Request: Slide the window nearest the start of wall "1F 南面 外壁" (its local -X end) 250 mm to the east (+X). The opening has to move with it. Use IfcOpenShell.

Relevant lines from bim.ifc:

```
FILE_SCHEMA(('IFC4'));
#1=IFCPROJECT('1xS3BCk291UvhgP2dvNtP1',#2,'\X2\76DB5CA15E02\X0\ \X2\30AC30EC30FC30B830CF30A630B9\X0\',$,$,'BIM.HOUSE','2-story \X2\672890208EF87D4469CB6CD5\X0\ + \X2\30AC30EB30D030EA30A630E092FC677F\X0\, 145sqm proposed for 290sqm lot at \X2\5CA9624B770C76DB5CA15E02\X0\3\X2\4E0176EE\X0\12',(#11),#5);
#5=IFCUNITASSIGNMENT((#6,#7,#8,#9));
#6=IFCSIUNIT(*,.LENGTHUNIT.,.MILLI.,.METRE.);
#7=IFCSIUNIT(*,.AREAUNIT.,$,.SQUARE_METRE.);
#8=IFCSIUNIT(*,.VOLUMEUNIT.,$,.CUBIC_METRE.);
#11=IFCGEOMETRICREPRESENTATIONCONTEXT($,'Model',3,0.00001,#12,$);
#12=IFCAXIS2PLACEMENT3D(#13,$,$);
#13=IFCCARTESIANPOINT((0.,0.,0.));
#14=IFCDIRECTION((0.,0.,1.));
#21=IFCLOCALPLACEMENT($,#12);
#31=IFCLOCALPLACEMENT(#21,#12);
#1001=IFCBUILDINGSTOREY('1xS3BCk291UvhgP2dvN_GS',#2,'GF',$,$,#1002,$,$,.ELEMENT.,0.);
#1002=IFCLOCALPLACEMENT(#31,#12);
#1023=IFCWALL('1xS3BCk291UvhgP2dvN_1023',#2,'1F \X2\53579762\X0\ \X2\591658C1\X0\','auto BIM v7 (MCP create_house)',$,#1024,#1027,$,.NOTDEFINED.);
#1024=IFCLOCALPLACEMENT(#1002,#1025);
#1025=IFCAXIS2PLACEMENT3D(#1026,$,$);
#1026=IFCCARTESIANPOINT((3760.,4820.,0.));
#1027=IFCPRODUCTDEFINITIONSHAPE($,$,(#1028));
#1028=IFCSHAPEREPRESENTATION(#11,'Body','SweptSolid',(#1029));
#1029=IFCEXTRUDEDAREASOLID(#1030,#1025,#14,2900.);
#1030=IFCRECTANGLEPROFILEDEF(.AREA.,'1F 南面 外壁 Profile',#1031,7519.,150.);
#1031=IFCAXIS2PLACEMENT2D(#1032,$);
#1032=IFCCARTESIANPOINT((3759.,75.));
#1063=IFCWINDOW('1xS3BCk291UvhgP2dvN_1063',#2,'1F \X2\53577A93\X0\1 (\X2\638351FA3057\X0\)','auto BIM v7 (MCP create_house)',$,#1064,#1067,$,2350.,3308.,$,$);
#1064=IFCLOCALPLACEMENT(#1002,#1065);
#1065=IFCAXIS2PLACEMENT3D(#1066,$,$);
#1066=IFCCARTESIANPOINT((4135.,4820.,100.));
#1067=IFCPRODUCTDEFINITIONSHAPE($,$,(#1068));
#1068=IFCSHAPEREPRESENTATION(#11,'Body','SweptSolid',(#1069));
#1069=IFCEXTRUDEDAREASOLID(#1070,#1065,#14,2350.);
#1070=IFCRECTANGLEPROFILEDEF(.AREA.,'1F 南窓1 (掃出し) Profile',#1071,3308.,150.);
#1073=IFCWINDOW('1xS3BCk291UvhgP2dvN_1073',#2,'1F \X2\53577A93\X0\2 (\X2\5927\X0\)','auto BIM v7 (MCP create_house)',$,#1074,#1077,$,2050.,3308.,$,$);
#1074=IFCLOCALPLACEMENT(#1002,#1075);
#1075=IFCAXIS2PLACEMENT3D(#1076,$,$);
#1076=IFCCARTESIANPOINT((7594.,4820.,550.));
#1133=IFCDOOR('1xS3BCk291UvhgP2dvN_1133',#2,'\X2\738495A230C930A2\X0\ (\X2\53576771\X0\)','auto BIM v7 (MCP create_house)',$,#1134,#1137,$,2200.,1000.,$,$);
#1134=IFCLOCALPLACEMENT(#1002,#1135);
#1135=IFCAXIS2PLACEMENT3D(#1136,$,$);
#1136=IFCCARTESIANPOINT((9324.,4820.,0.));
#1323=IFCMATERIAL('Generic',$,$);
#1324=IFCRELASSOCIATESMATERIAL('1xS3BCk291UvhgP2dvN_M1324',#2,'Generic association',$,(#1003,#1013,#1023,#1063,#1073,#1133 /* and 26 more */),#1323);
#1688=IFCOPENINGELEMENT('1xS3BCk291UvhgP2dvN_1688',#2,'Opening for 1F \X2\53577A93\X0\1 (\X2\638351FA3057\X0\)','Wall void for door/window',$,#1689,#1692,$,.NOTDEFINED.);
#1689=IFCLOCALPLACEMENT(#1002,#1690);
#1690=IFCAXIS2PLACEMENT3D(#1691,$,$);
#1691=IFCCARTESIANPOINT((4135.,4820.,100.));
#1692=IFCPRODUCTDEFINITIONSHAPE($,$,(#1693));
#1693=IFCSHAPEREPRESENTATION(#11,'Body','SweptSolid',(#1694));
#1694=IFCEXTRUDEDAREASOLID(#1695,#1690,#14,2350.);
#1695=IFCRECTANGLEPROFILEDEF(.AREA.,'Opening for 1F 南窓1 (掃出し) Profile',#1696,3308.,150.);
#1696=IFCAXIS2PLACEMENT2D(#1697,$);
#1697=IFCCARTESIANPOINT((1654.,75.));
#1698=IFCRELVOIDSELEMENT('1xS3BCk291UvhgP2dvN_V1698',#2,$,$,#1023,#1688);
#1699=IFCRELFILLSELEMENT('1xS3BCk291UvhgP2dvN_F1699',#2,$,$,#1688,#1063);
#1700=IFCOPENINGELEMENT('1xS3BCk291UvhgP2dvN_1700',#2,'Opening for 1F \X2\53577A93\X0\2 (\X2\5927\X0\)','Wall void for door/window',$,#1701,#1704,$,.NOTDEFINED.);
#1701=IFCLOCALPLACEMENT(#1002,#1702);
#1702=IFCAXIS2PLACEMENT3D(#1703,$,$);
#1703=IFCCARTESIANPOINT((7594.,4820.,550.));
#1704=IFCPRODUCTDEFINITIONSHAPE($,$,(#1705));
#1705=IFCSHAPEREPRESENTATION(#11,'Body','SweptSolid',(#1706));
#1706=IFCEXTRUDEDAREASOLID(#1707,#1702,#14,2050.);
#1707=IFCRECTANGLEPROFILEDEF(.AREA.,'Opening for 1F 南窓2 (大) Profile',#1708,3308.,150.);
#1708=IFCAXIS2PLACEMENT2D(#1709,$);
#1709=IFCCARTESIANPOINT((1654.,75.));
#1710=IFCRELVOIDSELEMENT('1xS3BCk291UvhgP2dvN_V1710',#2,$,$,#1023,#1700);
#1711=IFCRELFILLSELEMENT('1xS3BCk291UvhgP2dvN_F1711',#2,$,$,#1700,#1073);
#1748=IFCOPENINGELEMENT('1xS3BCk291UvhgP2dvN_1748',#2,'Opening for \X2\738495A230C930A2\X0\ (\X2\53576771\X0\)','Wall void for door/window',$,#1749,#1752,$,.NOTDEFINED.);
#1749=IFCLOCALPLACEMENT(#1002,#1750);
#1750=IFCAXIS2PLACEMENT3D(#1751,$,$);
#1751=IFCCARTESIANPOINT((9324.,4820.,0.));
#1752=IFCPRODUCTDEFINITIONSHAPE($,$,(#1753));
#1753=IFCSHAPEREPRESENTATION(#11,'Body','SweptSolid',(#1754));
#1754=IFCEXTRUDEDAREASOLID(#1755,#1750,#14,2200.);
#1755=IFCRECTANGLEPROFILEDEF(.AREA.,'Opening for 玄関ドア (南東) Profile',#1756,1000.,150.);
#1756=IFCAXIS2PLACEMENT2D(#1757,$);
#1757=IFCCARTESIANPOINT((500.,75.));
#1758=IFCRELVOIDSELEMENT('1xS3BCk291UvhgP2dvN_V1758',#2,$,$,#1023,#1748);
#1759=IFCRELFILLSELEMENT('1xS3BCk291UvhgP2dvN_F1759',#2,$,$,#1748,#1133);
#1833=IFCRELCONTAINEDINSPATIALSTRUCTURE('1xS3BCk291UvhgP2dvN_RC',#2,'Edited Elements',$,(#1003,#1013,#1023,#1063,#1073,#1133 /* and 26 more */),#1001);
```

```python
import ifcopenshell
import ifcopenshell.api.geometry
import ifcopenshell.util.placement

model = ifcopenshell.open("bim.ifc")

window = model.by_id(1063)
opening = window.FillsVoids[0].RelatingOpeningElement
wall = opening.VoidsElements[0].RelatingBuildingElement

wall_matrix = ifcopenshell.util.placement.get_local_placement(wall.ObjectPlacement)
shift = wall_matrix[:3, 0] * 250.0
before = ifcopenshell.util.placement.get_local_placement(window.ObjectPlacement)[:3, 3].copy()

# The window is not placed relative to its opening, so move both.
for product in (opening, window):
    matrix = ifcopenshell.util.placement.get_local_placement(product.ObjectPlacement)
    matrix[:3, 3] += shift
    ifcopenshell.api.geometry.edit_object_placement(model, product=product, matrix=matrix, is_si=False)

after = ifcopenshell.util.placement.get_local_placement(window.ObjectPlacement)[:3, 3]
print("window moved by", (after - before).round(3) + 0.0)

model.write("bim_rev.ifc")
```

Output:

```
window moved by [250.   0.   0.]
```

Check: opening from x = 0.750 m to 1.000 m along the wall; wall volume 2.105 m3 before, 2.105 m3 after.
